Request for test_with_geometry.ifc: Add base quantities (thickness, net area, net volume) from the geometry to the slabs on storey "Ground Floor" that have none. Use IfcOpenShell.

First a look at what the model holds.

```python
import ifcopenshell
import ifcopenshell.util.element
import ifcopenshell.util.unit

model = ifcopenshell.open("test_with_geometry.ifc")
print(model.schema)
for unit_type in ("LENGTHUNIT", "AREAUNIT", "VOLUMEUNIT"):
    print(unit_type, ifcopenshell.util.unit.calculate_unit_scale(model, unit_type))
storey = next(s for s in model.by_type("IfcBuildingStorey") if s.Name == "Ground Floor")
slabs = [e for e in ifcopenshell.util.element.get_decomposition(storey) if e.is_a("IfcSlab")]
for e in sorted(slabs, key=lambda e: e.id()):
    print(e.id(), e.is_a(), e.Name, list(ifcopenshell.util.element.get_psets(e, qtos_only=True)), sep=" | ")
```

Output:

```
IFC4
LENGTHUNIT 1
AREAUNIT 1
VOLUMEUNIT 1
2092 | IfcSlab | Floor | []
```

```python
import ifcopenshell
import ifcopenshell.api.pset
import ifcopenshell.geom
import ifcopenshell.util.element
import ifcopenshell.util.shape
import ifcopenshell.util.unit

model = ifcopenshell.open("test_with_geometry.ifc")
unit_scale = ifcopenshell.util.unit.calculate_unit_scale(model)
area_scale = ifcopenshell.util.unit.calculate_unit_scale(model, "AREAUNIT")
volume_scale = ifcopenshell.util.unit.calculate_unit_scale(model, "VOLUMEUNIT")
settings = ifcopenshell.geom.settings()

storey = next(s for s in model.by_type("IfcBuildingStorey") if s.Name == "Ground Floor")
slabs = [e for e in ifcopenshell.util.element.get_decomposition(storey) if e.is_a("IfcSlab")]

for e in sorted(slabs, key=lambda e: e.id()):
    if ifcopenshell.util.element.get_psets(e, qtos_only=True, should_inherit=False):
        continue
    # Geometry comes back in metres, in the element's own axes.
    shape = ifcopenshell.geom.create_shape(settings, e)
    values = {
        "Width": ifcopenshell.util.shape.get_z(shape.geometry) / unit_scale,
        "NetArea": ifcopenshell.util.shape.get_footprint_area(shape.geometry) / area_scale,
        "NetVolume": ifcopenshell.util.shape.get_volume(shape.geometry) / volume_scale,
    }
    qto = ifcopenshell.api.pset.add_qto(model, product=e, name="Qto_SlabBaseQuantities")
    ifcopenshell.api.pset.edit_qto(model, qto=qto, properties=values)
    print(e.id(), {k: round(v, 3) for k, v in values.items()})

model.write("test_with_geometry_updated.ifc")
```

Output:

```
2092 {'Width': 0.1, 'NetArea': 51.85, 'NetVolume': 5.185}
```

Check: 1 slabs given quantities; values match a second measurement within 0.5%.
